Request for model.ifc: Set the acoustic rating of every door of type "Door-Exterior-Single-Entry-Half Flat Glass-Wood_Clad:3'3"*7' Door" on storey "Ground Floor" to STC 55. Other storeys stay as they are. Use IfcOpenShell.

First a look at what the model holds.

```python
import ifcopenshell
import ifcopenshell.util.element

model = ifcopenshell.open("model.ifc")
print(model.schema)
storey = next(s for s in model.by_type("IfcBuildingStorey") if s.Name == "Ground Floor")
doors = [e for e in ifcopenshell.util.element.get_decomposition(storey) if e.is_a("IfcDoor")]
seen = {}
for e in doors:
    element_type = ifcopenshell.util.element.get_type(e)
    key = (element_type.Name if element_type != e and element_type else None, ifcopenshell.util.element.get_pset(e, "Pset_DoorCommon", "AcousticRating"))
    seen[key] = seen.get(key, 0) + 1
for (name, value), count in sorted(seen.items(), key=str):
    print(count, "x", name, "|", value)
```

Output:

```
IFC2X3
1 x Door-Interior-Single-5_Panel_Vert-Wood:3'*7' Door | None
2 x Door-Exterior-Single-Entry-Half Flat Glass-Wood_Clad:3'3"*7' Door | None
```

```python
import ifcopenshell
import ifcopenshell.api.pset
import ifcopenshell.util.element

model = ifcopenshell.open("model.ifc")

storey = next(s for s in model.by_type("IfcBuildingStorey") if s.Name == "Ground Floor")
doors = [e for e in ifcopenshell.util.element.get_decomposition(storey) if e.is_a("IfcDoor")]

count = 0
for e in doors:
    element_type = ifcopenshell.util.element.get_type(e)
    if element_type in (None, e) or element_type.Name != 'Door-Exterior-Single-Entry-Half Flat Glass-Wood_Clad:3\'3"*7\' Door':
        continue
    # add_pset returns the element's existing set when there is one.
    pset = ifcopenshell.api.pset.add_pset(model, product=e, name="Pset_DoorCommon")
    ifcopenshell.api.pset.edit_pset(model, pset=pset, properties={"AcousticRating": "STC 55"})
    count += 1

print(count, "doors updated")

model.write("model_updated.ifc")
```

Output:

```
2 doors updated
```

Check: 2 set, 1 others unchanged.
